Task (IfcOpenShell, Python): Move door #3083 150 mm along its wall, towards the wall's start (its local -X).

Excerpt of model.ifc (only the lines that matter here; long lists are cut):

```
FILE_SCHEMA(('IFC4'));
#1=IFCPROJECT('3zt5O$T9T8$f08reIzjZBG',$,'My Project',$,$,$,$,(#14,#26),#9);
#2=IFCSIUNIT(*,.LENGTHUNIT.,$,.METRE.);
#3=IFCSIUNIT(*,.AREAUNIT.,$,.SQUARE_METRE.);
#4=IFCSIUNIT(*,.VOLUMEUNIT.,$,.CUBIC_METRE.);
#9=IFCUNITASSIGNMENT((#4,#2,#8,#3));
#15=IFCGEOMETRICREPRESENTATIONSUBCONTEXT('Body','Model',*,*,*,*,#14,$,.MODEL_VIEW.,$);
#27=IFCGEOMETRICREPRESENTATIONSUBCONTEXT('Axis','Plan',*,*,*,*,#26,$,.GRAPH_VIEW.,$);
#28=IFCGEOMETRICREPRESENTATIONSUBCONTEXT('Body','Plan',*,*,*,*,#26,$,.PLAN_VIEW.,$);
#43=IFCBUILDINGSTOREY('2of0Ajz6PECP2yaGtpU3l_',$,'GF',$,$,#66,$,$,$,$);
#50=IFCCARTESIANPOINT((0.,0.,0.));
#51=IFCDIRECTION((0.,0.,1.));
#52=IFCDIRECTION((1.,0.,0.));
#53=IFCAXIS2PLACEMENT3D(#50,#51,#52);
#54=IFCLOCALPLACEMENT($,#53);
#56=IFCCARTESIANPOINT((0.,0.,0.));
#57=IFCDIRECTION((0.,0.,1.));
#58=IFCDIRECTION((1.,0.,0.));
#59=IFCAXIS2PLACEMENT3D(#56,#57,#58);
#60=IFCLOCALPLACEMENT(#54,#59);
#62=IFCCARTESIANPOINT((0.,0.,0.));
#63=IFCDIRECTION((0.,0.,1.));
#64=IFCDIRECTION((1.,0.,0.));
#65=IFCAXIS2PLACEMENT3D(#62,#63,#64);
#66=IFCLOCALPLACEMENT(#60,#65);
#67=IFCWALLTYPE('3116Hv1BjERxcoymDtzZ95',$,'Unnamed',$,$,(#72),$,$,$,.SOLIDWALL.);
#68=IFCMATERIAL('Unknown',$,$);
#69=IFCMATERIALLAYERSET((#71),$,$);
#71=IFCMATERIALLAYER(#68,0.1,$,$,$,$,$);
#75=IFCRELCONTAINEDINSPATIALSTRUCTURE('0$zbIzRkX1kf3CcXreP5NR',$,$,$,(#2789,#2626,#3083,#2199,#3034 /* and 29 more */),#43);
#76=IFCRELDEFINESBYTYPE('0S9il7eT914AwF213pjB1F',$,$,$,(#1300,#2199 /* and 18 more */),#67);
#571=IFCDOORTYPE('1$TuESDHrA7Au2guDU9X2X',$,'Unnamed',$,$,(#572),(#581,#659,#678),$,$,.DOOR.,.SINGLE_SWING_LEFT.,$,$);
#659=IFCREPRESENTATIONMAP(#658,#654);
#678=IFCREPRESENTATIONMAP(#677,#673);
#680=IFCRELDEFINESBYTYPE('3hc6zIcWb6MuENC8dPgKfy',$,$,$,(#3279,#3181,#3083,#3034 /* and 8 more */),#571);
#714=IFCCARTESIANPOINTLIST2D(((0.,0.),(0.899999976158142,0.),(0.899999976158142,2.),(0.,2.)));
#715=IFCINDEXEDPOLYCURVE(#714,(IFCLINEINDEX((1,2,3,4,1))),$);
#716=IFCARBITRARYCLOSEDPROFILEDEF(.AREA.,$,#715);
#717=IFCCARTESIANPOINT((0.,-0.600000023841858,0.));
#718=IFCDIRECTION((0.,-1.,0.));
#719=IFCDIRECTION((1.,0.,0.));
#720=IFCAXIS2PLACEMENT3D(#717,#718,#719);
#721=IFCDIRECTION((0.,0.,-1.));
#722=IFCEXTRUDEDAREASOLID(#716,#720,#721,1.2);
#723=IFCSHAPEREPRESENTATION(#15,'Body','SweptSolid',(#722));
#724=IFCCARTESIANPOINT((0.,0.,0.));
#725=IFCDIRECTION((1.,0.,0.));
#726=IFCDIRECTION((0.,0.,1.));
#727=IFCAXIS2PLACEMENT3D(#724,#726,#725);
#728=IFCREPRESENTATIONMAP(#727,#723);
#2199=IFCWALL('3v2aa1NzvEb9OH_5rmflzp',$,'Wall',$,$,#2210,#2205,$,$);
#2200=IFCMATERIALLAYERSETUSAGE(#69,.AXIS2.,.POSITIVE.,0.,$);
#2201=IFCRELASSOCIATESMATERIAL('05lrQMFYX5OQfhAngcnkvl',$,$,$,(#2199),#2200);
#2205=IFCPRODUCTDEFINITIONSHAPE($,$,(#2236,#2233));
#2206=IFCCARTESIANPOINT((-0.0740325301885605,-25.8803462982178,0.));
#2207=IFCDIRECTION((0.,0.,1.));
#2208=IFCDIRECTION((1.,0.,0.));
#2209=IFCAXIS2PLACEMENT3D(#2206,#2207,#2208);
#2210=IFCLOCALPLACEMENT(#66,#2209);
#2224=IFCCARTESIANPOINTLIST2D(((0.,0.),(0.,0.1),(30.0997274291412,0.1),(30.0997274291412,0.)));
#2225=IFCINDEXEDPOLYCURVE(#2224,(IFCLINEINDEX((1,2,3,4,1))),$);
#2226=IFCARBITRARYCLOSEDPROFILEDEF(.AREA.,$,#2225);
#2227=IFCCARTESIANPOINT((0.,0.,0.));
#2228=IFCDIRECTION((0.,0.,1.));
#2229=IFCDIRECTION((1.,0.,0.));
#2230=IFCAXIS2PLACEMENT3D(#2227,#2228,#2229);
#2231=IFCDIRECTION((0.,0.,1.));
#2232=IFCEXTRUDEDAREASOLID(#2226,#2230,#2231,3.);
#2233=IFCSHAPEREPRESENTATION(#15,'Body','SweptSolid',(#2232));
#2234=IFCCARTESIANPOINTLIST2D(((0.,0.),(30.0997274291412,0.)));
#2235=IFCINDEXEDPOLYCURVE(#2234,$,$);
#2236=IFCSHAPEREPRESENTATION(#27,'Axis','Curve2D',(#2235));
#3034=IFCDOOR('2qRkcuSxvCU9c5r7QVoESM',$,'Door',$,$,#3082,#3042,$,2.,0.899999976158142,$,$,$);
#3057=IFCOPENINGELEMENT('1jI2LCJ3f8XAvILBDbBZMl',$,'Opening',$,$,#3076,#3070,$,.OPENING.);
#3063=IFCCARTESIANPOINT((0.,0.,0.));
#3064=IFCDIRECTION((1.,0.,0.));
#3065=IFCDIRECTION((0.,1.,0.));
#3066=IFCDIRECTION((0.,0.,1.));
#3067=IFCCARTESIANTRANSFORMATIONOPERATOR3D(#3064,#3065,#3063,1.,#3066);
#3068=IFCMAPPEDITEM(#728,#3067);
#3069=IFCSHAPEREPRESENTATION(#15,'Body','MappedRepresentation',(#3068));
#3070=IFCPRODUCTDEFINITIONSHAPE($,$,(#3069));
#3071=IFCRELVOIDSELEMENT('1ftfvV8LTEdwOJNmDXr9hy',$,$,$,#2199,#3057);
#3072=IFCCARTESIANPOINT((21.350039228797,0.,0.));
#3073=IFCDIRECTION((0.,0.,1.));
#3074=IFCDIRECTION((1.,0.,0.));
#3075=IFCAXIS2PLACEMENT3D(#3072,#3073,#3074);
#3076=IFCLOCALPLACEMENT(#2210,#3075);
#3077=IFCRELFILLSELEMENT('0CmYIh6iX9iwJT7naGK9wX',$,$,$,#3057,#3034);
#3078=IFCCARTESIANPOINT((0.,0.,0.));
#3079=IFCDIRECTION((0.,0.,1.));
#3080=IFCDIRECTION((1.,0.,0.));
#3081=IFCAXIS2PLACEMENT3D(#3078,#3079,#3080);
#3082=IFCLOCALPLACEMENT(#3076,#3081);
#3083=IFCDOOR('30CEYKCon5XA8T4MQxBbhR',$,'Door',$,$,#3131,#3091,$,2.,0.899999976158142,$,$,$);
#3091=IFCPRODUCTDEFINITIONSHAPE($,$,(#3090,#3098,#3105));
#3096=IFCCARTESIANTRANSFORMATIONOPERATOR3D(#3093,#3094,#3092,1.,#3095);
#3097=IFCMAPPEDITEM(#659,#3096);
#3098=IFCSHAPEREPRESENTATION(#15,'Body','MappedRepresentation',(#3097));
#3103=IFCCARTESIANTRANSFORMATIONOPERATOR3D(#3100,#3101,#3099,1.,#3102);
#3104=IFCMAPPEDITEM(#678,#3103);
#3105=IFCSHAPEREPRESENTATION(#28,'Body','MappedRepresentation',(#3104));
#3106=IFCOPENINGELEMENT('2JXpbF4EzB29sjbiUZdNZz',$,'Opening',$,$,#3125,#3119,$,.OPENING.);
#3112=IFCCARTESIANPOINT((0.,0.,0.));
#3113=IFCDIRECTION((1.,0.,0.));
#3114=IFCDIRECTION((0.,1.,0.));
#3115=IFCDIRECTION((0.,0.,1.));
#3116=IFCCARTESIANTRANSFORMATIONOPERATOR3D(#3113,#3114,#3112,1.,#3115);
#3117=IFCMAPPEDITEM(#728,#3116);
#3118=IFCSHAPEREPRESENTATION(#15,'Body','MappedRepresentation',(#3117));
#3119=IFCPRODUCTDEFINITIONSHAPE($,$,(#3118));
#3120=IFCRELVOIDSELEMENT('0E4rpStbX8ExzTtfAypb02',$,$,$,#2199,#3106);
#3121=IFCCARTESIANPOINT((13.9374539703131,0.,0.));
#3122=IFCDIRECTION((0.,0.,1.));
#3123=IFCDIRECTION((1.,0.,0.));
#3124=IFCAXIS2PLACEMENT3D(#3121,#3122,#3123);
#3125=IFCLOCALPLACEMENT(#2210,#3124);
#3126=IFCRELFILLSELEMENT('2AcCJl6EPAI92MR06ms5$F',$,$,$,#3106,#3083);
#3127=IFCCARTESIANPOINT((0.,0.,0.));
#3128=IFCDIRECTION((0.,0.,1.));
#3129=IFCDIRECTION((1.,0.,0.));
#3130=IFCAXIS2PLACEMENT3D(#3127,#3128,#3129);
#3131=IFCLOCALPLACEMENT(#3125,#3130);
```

```python
import ifcopenshell
import ifcopenshell.api.geometry
import ifcopenshell.util.placement
import ifcopenshell.util.unit

model = ifcopenshell.open("model.ifc")
unit_scale = ifcopenshell.util.unit.calculate_unit_scale(model)

door = model.by_guid("30CEYKCon5XA8T4MQxBbhR")
opening = door.FillsVoids[0].RelatingOpeningElement
wall = opening.VoidsElements[0].RelatingBuildingElement

wall_matrix = ifcopenshell.util.placement.get_local_placement(wall.ObjectPlacement)
shift = wall_matrix[:3, 0] * -0.15 / unit_scale
before = ifcopenshell.util.placement.get_local_placement(door.ObjectPlacement)[:3, 3].copy()

# The door is placed relative to its opening, so it follows when the opening moves.
matrix = ifcopenshell.util.placement.get_local_placement(opening.ObjectPlacement)
matrix[:3, 3] += shift
ifcopenshell.api.geometry.edit_object_placement(
    model, product=opening, matrix=matrix, is_si=False, should_transform_children=True
)

after = ifcopenshell.util.placement.get_local_placement(door.ObjectPlacement)[:3, 3]
print("door moved by", (after - before).round(3) + 0.0)

model.write("model-out.ifc")
```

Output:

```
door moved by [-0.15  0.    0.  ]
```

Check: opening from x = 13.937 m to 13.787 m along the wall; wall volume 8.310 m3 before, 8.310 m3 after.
